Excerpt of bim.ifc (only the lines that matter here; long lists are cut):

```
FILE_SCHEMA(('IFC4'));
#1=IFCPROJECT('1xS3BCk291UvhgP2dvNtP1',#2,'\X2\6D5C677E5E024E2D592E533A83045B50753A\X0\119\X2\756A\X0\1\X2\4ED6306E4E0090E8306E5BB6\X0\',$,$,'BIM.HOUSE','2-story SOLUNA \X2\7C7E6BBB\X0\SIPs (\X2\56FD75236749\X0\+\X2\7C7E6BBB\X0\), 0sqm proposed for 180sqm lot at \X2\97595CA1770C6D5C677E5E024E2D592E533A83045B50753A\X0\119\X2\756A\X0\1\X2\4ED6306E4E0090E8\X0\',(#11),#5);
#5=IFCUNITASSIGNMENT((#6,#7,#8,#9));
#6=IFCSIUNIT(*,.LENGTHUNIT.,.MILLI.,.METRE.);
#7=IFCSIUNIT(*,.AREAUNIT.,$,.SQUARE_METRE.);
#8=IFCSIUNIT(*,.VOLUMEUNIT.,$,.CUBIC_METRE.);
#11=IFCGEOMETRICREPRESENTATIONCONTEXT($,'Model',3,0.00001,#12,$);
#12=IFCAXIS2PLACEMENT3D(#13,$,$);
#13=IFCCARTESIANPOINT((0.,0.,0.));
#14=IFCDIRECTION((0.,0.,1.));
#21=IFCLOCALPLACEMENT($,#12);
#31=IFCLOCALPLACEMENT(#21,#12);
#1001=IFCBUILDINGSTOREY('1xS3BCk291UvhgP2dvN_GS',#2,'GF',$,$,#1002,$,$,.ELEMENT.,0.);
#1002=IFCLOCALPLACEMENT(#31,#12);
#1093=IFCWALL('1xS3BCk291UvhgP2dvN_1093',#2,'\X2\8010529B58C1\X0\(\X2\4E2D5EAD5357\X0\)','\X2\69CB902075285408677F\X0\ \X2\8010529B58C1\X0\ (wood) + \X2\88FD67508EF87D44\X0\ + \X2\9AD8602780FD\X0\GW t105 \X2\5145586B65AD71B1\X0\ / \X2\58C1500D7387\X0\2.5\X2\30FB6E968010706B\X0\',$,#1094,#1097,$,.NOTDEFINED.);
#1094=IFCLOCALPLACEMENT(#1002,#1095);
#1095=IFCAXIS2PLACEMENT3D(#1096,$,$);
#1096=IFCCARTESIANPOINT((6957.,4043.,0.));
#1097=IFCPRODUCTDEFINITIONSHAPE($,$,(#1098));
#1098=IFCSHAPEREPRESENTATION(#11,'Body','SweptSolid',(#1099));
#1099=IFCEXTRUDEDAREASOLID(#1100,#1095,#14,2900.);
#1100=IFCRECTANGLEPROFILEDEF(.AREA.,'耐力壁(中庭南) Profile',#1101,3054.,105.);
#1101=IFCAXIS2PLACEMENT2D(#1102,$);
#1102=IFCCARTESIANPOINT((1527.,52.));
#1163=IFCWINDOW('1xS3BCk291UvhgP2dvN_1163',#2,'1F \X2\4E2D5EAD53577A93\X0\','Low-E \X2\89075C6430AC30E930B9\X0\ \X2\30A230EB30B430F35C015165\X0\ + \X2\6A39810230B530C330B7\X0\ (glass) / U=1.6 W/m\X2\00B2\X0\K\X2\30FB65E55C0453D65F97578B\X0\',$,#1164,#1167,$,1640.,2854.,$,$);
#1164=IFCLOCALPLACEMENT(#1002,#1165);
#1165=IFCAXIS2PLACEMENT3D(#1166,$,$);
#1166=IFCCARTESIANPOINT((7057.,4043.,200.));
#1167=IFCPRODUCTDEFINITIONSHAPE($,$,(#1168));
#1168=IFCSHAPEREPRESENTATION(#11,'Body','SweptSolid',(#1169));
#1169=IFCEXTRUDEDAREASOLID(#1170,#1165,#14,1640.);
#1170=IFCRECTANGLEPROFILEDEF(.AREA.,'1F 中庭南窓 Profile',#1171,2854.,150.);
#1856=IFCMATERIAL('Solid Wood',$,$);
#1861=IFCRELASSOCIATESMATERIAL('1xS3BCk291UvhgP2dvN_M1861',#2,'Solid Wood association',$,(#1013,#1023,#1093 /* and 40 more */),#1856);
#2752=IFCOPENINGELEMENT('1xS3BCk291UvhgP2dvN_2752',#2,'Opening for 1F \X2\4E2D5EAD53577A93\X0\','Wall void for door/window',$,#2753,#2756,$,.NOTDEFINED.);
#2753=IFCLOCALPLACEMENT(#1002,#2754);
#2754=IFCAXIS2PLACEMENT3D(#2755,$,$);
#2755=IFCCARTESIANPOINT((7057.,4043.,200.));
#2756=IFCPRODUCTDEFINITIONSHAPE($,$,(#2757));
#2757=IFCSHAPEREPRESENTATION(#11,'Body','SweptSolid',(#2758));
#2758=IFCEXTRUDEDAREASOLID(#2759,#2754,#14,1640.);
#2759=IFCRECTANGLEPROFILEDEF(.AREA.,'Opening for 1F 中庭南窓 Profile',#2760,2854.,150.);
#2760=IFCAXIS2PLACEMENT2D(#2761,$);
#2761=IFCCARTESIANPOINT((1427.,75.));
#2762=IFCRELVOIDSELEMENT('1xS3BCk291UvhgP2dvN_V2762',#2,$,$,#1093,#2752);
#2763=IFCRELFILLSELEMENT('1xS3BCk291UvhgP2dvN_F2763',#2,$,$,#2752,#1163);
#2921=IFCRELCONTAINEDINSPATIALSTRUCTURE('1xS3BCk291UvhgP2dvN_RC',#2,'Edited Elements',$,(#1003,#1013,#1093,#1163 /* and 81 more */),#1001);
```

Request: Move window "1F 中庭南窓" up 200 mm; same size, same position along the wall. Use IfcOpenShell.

```python
import numpy as np
import ifcopenshell
import ifcopenshell.api.geometry
import ifcopenshell.util.placement
import ifcopenshell.util.unit

model = ifcopenshell.open("bim.ifc")
unit_scale = ifcopenshell.util.unit.calculate_unit_scale(model)

window = model.by_guid("1xS3BCk291UvhgP2dvN_1163")
opening = window.FillsVoids[0].RelatingOpeningElement
dz = 200.0

shift = np.array([0.0, 0.0, dz])
# The window is not placed relative to its opening, so move both.
for product in (opening, window):
    matrix = ifcopenshell.util.placement.get_local_placement(product.ObjectPlacement)
    matrix[:3, 3] += shift
    ifcopenshell.api.geometry.edit_object_placement(model, product=product, matrix=matrix, is_si=False)

print(f"moved by {dz * unit_scale:+.3f} m")

model.write("bim_edited.ifc")
```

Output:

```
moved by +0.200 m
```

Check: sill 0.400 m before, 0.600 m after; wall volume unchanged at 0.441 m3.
